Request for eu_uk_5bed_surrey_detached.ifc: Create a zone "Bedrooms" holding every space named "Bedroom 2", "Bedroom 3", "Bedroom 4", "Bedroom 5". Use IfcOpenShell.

First a look at what the model holds.

```python
import ifcopenshell

model = ifcopenshell.open("eu_uk_5bed_surrey_detached.ifc")
print(model.schema)
seen = {}
for space in model.by_type("IfcSpace"):
    seen[space.LongName] = seen.get(space.LongName, 0) + 1
for name, count in sorted(seen.items(), key=str):
    print(count, "x", name)
print("zones:", [z.Name for z in model.by_type("IfcZone")][:20])
```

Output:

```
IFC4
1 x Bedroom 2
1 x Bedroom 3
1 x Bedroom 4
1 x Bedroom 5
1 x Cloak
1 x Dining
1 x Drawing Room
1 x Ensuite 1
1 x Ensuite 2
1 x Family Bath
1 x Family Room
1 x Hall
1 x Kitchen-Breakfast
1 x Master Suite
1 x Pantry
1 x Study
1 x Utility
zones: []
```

```python
import ifcopenshell
import ifcopenshell.api.group
import ifcopenshell.api.root

model = ifcopenshell.open("eu_uk_5bed_surrey_detached.ifc")

names = {"Bedroom 2", "Bedroom 3", "Bedroom 4", "Bedroom 5"}
spaces = [s for s in model.by_type("IfcSpace") if s.LongName in names]

zone = ifcopenshell.api.root.create_entity(model, ifc_class="IfcZone", name="Bedrooms")
ifcopenshell.api.group.assign_group(model, products=spaces, group=zone)
print(len(spaces), "spaces in", zone.Name)

model.write("eu_uk_5bed_surrey_detached-out.ifc")
```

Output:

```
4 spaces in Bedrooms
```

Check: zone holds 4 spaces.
